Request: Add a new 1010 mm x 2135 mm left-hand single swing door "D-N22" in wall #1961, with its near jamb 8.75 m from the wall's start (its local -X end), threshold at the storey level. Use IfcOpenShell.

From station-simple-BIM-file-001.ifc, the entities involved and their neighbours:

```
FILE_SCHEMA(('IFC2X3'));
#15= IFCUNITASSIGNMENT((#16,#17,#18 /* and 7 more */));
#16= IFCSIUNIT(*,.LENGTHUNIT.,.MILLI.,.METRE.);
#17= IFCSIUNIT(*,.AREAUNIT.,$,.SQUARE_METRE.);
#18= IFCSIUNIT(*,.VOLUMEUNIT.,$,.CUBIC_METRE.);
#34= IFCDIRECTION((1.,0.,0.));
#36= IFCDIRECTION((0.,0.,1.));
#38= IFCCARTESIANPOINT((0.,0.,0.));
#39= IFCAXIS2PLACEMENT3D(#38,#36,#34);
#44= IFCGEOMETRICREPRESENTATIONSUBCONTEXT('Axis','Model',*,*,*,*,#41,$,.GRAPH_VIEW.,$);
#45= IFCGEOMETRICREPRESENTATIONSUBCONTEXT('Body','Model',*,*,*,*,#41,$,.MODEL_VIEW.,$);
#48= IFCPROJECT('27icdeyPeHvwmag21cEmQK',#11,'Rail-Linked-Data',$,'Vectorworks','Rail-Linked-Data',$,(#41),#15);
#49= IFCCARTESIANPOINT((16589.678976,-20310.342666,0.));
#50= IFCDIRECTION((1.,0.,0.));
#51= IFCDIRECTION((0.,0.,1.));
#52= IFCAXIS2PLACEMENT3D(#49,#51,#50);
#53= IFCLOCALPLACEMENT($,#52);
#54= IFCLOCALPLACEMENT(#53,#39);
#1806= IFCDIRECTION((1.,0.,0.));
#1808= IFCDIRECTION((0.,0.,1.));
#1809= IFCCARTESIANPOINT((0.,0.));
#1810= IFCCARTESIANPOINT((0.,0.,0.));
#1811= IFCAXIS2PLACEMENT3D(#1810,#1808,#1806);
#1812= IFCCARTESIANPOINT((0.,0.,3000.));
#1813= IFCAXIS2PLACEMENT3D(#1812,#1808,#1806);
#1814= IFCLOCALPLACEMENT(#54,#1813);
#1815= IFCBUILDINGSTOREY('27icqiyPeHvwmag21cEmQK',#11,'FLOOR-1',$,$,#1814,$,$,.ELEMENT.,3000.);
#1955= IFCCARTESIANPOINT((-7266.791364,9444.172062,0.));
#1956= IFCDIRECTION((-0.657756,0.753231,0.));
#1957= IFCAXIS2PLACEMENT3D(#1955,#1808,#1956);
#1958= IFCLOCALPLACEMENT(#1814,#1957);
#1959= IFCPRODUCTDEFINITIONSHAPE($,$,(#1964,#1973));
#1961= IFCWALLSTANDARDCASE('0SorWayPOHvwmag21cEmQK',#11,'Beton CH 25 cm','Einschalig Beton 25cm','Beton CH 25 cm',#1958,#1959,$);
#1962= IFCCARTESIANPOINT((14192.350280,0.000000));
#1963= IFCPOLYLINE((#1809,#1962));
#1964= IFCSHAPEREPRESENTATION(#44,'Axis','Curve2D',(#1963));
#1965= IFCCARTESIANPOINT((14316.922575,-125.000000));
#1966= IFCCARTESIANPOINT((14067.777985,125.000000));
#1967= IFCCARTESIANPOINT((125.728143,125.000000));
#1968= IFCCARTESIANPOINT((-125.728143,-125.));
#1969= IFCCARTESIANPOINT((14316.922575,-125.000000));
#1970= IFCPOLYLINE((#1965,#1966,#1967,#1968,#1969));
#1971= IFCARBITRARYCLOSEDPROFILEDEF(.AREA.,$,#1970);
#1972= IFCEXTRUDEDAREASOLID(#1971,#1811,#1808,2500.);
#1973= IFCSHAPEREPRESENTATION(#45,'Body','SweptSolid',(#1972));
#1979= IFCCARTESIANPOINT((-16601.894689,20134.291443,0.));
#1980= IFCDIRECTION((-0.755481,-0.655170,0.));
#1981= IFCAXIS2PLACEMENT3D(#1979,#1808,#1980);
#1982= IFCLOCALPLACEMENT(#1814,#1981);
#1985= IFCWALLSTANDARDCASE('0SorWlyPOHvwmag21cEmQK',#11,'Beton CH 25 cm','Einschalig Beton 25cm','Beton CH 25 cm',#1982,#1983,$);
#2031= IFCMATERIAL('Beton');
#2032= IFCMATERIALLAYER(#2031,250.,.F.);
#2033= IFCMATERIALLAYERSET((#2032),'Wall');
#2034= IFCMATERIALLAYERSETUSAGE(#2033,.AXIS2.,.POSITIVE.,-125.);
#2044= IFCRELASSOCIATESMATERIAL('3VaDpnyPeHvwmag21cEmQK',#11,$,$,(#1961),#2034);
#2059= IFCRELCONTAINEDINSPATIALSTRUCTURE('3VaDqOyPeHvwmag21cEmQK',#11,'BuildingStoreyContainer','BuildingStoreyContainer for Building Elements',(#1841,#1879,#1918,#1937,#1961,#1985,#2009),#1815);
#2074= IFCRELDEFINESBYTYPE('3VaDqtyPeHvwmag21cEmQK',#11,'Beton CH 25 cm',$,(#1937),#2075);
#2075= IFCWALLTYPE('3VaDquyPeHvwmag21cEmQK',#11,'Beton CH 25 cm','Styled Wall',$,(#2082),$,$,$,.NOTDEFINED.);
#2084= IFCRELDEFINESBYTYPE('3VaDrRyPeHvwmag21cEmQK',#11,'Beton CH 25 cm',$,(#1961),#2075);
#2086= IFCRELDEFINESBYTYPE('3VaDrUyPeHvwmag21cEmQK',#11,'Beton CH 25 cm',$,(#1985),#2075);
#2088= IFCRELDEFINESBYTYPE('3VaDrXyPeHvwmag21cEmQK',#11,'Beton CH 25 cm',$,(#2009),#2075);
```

```python
import numpy as np
import ifcopenshell
import ifcopenshell.api.feature
import ifcopenshell.api.geometry
import ifcopenshell.api.root
import ifcopenshell.api.spatial
import ifcopenshell.api.type
import ifcopenshell.geom
import ifcopenshell.util.element
import ifcopenshell.util.placement
import ifcopenshell.util.representation
import ifcopenshell.util.shape
import ifcopenshell.util.unit

model = ifcopenshell.open("station-simple-BIM-file-001.ifc")
unit_scale = ifcopenshell.util.unit.calculate_unit_scale(model)
settings = ifcopenshell.geom.settings()


def volume(element):
    """Net volume in cubic metres, openings subtracted."""
    shape = ifcopenshell.geom.create_shape(settings, element)
    return ifcopenshell.util.shape.get_volume(shape.geometry)


wall = model.by_guid("0SorWayPOHvwmag21cEmQK")
storey = ifcopenshell.util.element.get_container(wall, ifc_class="IfcBuildingStorey")
context = ifcopenshell.util.representation.get_context(model, "Model", "Body", "MODEL_VIEW")
before = volume(wall)

width, height, from_end, sill = 1.01, 2.135, 8.75, 0.0  # metres

# The wall runs along its own X axis, and the end named is its -X end.
wall_shape = ifcopenshell.geom.create_shape(settings, wall)
x, y, z = ifcopenshell.util.shape.get_vertices(wall_shape.geometry).T
start = x.min() + from_end
face, thickness = float(y.min()), float(y.max() - y.min())
wall_matrix = ifcopenshell.util.placement.get_local_placement(wall.ObjectPlacement)
level = ifcopenshell.util.placement.get_local_placement(storey.ObjectPlacement)[2, 3]


def in_wall(x, y):
    """Placement at x, y metres in the wall's axes, at sill height."""
    matrix = wall_matrix.copy()
    matrix[:, 3] = wall_matrix @ np.array([x / unit_scale, y / unit_scale, 0.0, 1.0])
    matrix[2, 3] = level + sill / unit_scale
    return matrix


# Opening: a box that overshoots both wall faces by 50 mm.
opening = ifcopenshell.api.root.create_entity(model, ifc_class="IfcOpeningElement")
box = ifcopenshell.api.geometry.add_wall_representation(
    model, context=context, length=width, height=height, thickness=thickness + 0.1
)
ifcopenshell.api.geometry.assign_representation(model, product=opening, representation=box)
ifcopenshell.api.geometry.edit_object_placement(model, product=opening, matrix=in_wall(start, face - 0.05), is_si=False)
ifcopenshell.api.feature.add_feature(model, feature=opening, element=wall)

door = ifcopenshell.api.root.create_entity(model, ifc_class="IfcDoor", name="D-N22")
door.OverallWidth, door.OverallHeight = width / unit_scale, height / unit_scale
body = ifcopenshell.api.geometry.add_door_representation(
    model,
    context=context,
    overall_width=door.OverallWidth,
    overall_height=door.OverallHeight,
    operation_type="SINGLE_SWING_LEFT",
    lining_properties={"LiningDepth": thickness / unit_scale, "ThresholdDepth": thickness / unit_scale},
)
ifcopenshell.api.geometry.assign_representation(model, product=door, representation=body)
ifcopenshell.api.spatial.assign_container(model, products=[door], relating_structure=storey)
fills = ifcopenshell.api.feature.add_filling(model, opening=opening, element=door)
fills.OwnerHistory = door.OwnerHistory  # required in IFC2X3

# IFC2X3 keeps the operation on the door style.
style = ifcopenshell.api.root.create_entity(model, ifc_class="IfcDoorStyle", name="D-N22")
style.OperationType, style.ConstructionType = "SINGLE_SWING_LEFT", "NOTDEFINED"
style.ParameterTakesPrecedence = style.Sizeable = False
ifcopenshell.api.type.assign_type(model, related_objects=[door], relating_type=style)

# The lining spans the wall, so the door starts at the wall face.
ifcopenshell.api.geometry.edit_object_placement(model, product=door, matrix=in_wall(start, face), is_si=False)

after = volume(wall)

print(f"wall volume {before:.3f} -> {after:.3f} m3")

model.write("station-simple-BIM-file-001_updated.ifc")
```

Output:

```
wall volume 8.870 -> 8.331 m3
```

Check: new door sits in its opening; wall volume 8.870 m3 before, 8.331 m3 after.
